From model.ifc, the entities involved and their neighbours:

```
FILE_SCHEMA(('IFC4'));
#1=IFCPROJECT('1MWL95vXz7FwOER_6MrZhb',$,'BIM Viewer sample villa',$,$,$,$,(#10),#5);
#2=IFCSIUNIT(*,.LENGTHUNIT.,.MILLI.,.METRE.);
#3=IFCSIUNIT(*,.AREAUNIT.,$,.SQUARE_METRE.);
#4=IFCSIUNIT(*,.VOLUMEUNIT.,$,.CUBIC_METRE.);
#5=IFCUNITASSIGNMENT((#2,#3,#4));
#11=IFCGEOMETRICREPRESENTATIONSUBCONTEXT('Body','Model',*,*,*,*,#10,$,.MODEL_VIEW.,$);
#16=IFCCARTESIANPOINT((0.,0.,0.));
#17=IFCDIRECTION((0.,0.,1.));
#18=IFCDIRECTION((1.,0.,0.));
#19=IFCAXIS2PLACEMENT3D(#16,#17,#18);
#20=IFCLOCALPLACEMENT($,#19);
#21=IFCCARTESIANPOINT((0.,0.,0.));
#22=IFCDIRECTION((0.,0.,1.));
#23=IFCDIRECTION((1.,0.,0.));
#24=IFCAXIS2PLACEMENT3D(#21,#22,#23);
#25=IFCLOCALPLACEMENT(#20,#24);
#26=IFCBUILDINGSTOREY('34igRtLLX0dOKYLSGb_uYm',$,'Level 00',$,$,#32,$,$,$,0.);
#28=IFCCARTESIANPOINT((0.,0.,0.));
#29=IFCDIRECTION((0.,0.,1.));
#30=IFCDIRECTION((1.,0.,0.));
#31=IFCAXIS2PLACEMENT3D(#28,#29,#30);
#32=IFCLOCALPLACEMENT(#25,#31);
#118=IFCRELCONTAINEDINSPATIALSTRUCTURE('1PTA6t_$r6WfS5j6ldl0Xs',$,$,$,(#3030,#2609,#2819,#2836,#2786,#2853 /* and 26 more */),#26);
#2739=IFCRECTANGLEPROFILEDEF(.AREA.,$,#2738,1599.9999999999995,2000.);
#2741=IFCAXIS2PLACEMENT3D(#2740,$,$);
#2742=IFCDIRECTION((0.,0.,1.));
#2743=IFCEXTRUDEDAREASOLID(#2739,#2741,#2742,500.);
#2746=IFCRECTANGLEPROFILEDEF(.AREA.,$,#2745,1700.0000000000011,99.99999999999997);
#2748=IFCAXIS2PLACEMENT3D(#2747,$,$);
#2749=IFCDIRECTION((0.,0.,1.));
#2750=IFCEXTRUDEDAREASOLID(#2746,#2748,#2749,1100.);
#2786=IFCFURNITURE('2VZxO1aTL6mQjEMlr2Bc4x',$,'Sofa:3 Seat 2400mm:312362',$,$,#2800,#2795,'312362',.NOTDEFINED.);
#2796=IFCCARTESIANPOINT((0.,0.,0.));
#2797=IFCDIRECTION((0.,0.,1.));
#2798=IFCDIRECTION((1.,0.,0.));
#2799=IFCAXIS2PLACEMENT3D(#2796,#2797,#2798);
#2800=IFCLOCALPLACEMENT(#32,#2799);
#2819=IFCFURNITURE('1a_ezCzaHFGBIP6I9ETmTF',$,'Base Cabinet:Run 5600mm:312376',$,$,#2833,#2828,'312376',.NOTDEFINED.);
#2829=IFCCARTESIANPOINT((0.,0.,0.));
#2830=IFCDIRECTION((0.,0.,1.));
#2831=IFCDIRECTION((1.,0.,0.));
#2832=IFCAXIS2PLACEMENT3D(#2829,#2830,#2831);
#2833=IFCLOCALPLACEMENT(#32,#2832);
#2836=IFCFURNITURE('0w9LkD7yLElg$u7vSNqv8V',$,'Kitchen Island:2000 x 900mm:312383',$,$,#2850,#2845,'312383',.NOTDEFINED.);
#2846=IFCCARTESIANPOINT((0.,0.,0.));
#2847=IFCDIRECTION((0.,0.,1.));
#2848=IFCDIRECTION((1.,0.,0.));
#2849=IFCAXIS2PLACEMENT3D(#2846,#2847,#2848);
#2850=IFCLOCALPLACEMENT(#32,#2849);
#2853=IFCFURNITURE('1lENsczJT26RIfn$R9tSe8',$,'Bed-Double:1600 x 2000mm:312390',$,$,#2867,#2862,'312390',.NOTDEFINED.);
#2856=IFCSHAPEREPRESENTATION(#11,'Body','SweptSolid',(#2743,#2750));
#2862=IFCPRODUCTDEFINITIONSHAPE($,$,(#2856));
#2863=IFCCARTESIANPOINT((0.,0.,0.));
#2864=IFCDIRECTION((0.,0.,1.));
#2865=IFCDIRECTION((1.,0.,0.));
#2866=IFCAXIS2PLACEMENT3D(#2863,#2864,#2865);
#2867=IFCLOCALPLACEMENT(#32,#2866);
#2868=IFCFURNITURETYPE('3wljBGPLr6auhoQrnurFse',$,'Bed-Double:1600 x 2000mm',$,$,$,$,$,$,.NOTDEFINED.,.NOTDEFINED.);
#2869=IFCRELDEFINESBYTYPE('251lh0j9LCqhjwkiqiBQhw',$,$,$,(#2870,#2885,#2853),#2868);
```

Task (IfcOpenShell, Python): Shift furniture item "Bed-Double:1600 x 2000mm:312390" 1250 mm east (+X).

```python
import ifcopenshell
import ifcopenshell.api.geometry
import ifcopenshell.util.placement

model = ifcopenshell.open("model.ifc")

item = model.by_guid("1lENsczJT26RIfn$R9tSe8")
matrix = ifcopenshell.util.placement.get_local_placement(item.ObjectPlacement)
matrix[0, 3] += 1250.0
ifcopenshell.api.geometry.edit_object_placement(model, product=item, matrix=matrix, is_si=False)

print(ifcopenshell.util.placement.get_local_placement(item.ObjectPlacement).round(3) + 0.0)

model.write("model_edited.ifc")
```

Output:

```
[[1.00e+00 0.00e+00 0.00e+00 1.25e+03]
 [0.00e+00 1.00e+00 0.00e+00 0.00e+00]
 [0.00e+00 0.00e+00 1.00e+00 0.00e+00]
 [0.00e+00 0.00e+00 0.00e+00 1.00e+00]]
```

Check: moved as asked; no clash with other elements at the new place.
